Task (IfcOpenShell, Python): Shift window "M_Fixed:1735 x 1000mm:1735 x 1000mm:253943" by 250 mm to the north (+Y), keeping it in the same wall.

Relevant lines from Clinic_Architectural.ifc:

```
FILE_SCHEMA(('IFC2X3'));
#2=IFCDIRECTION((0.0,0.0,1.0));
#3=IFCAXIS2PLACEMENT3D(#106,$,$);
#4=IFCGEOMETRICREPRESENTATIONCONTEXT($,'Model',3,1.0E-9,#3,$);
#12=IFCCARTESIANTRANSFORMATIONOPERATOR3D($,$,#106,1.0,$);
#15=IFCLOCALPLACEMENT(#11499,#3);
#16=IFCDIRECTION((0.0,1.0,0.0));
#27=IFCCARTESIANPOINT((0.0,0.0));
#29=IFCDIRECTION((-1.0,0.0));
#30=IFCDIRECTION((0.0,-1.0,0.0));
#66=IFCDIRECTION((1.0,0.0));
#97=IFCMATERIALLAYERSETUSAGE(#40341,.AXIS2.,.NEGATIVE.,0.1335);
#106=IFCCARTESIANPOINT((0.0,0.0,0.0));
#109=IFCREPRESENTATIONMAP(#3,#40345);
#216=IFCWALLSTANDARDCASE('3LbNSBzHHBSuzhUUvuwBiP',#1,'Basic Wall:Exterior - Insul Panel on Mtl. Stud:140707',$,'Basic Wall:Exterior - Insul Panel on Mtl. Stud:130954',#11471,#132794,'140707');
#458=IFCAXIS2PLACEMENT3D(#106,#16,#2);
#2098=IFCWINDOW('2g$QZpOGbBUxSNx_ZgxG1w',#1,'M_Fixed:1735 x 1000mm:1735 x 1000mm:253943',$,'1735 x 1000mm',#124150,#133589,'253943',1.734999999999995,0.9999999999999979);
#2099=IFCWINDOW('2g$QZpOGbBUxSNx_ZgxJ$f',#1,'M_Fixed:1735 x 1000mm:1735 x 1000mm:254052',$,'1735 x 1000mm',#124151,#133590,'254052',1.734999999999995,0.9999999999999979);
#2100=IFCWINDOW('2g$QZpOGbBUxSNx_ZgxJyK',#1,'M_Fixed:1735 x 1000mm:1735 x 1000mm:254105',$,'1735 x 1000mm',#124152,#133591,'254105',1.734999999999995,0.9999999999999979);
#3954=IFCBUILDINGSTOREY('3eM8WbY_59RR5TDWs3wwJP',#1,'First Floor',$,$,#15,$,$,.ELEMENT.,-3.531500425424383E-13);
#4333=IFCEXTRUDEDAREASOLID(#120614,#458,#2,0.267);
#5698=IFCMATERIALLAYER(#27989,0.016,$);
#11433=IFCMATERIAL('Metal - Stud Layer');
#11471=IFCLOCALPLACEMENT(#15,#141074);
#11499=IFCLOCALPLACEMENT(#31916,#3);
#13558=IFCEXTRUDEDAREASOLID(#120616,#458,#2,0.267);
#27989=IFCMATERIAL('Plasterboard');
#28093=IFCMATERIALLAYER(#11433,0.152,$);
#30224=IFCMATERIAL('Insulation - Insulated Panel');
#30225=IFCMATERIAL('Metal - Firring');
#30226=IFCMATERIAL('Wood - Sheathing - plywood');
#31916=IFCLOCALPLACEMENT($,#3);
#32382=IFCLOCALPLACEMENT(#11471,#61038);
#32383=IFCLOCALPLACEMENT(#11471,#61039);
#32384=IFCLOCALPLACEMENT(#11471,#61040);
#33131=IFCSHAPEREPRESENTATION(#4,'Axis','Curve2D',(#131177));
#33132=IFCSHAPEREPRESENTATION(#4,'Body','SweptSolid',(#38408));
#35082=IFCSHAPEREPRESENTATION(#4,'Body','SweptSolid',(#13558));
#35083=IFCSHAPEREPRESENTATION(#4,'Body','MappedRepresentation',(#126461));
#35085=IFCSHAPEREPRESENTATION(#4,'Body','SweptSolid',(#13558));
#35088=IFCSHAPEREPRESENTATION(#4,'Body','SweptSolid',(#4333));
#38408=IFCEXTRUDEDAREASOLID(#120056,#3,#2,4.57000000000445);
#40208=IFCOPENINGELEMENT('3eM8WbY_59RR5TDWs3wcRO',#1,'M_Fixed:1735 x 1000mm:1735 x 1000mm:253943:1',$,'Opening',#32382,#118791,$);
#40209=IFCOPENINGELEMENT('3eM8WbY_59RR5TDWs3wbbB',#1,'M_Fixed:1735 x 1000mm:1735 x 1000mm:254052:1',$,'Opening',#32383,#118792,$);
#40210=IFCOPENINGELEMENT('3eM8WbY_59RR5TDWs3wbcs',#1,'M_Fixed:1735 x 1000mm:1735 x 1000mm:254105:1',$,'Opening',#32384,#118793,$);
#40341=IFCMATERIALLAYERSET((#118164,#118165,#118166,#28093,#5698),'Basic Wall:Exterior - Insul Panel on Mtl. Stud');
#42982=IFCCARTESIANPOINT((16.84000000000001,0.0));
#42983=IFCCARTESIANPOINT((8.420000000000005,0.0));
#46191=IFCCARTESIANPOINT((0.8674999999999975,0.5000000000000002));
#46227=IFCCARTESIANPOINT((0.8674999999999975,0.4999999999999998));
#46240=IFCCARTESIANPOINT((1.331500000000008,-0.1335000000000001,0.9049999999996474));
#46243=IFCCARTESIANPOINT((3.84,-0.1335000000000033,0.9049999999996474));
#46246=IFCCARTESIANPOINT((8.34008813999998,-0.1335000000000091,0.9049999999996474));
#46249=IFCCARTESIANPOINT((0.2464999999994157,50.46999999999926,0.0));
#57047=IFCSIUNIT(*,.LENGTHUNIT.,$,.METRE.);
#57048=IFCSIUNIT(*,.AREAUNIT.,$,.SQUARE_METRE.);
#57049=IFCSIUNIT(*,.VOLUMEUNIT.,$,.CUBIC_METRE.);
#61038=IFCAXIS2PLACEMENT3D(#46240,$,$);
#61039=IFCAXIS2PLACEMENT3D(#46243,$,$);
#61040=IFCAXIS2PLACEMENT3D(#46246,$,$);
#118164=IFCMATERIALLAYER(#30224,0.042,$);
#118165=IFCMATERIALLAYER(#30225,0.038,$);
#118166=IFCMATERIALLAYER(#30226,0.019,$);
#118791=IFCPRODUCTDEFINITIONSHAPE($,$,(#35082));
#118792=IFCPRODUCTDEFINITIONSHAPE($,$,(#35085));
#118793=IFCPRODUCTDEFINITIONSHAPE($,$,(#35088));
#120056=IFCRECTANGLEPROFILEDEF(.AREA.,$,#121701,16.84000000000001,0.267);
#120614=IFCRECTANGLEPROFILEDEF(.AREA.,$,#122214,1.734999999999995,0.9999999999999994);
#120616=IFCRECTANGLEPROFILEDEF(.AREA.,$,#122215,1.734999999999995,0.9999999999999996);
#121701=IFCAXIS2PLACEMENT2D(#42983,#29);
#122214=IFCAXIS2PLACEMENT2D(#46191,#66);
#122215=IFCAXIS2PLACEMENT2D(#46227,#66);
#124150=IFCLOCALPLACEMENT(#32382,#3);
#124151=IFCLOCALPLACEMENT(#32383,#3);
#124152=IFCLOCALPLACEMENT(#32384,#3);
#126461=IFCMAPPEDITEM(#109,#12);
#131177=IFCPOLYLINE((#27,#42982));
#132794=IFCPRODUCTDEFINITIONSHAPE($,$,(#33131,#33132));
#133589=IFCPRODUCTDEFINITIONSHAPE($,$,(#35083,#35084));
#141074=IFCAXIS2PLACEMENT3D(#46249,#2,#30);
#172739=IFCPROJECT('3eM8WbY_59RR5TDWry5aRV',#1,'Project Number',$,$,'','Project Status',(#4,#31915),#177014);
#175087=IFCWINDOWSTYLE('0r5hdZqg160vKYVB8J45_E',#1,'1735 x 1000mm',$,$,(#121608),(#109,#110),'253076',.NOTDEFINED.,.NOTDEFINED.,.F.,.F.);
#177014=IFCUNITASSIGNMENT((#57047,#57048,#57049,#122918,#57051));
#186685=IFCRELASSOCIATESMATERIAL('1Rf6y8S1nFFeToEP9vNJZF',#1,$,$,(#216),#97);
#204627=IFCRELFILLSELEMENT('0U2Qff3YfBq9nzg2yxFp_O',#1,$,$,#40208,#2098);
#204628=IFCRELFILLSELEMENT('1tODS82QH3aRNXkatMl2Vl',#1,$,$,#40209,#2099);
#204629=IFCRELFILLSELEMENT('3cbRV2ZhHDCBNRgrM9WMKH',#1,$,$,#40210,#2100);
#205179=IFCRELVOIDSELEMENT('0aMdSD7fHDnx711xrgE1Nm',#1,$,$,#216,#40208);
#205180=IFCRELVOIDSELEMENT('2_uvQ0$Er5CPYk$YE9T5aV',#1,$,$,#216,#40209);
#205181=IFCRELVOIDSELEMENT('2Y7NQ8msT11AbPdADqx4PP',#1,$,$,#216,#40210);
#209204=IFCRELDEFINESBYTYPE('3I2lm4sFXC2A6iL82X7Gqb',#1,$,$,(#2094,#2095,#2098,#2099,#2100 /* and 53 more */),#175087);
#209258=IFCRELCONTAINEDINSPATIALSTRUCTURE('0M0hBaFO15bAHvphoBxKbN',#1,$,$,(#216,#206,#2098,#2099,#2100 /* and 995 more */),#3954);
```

```python
import ifcopenshell
import ifcopenshell.api.geometry
import ifcopenshell.util.placement
import ifcopenshell.util.unit

model = ifcopenshell.open("Clinic_Architectural.ifc")
unit_scale = ifcopenshell.util.unit.calculate_unit_scale(model)

window = model.by_id(2098)
opening = window.FillsVoids[0].RelatingOpeningElement
wall = opening.VoidsElements[0].RelatingBuildingElement

wall_matrix = ifcopenshell.util.placement.get_local_placement(wall.ObjectPlacement)
shift = wall_matrix[:3, 0] * -0.25 / unit_scale
before = ifcopenshell.util.placement.get_local_placement(window.ObjectPlacement)[:3, 3].copy()

# The window is placed relative to its opening, so it follows when the opening moves.
matrix = ifcopenshell.util.placement.get_local_placement(opening.ObjectPlacement)
matrix[:3, 3] += shift
ifcopenshell.api.geometry.edit_object_placement(
    model, product=opening, matrix=matrix, is_si=False, should_transform_children=True
)

after = ifcopenshell.util.placement.get_local_placement(window.ObjectPlacement)[:3, 3]
print("window moved by", (after - before).round(3) + 0.0)

model.write("Clinic_Architectural_rev.ifc")
```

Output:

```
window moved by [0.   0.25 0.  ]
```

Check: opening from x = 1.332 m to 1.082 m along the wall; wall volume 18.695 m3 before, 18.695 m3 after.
